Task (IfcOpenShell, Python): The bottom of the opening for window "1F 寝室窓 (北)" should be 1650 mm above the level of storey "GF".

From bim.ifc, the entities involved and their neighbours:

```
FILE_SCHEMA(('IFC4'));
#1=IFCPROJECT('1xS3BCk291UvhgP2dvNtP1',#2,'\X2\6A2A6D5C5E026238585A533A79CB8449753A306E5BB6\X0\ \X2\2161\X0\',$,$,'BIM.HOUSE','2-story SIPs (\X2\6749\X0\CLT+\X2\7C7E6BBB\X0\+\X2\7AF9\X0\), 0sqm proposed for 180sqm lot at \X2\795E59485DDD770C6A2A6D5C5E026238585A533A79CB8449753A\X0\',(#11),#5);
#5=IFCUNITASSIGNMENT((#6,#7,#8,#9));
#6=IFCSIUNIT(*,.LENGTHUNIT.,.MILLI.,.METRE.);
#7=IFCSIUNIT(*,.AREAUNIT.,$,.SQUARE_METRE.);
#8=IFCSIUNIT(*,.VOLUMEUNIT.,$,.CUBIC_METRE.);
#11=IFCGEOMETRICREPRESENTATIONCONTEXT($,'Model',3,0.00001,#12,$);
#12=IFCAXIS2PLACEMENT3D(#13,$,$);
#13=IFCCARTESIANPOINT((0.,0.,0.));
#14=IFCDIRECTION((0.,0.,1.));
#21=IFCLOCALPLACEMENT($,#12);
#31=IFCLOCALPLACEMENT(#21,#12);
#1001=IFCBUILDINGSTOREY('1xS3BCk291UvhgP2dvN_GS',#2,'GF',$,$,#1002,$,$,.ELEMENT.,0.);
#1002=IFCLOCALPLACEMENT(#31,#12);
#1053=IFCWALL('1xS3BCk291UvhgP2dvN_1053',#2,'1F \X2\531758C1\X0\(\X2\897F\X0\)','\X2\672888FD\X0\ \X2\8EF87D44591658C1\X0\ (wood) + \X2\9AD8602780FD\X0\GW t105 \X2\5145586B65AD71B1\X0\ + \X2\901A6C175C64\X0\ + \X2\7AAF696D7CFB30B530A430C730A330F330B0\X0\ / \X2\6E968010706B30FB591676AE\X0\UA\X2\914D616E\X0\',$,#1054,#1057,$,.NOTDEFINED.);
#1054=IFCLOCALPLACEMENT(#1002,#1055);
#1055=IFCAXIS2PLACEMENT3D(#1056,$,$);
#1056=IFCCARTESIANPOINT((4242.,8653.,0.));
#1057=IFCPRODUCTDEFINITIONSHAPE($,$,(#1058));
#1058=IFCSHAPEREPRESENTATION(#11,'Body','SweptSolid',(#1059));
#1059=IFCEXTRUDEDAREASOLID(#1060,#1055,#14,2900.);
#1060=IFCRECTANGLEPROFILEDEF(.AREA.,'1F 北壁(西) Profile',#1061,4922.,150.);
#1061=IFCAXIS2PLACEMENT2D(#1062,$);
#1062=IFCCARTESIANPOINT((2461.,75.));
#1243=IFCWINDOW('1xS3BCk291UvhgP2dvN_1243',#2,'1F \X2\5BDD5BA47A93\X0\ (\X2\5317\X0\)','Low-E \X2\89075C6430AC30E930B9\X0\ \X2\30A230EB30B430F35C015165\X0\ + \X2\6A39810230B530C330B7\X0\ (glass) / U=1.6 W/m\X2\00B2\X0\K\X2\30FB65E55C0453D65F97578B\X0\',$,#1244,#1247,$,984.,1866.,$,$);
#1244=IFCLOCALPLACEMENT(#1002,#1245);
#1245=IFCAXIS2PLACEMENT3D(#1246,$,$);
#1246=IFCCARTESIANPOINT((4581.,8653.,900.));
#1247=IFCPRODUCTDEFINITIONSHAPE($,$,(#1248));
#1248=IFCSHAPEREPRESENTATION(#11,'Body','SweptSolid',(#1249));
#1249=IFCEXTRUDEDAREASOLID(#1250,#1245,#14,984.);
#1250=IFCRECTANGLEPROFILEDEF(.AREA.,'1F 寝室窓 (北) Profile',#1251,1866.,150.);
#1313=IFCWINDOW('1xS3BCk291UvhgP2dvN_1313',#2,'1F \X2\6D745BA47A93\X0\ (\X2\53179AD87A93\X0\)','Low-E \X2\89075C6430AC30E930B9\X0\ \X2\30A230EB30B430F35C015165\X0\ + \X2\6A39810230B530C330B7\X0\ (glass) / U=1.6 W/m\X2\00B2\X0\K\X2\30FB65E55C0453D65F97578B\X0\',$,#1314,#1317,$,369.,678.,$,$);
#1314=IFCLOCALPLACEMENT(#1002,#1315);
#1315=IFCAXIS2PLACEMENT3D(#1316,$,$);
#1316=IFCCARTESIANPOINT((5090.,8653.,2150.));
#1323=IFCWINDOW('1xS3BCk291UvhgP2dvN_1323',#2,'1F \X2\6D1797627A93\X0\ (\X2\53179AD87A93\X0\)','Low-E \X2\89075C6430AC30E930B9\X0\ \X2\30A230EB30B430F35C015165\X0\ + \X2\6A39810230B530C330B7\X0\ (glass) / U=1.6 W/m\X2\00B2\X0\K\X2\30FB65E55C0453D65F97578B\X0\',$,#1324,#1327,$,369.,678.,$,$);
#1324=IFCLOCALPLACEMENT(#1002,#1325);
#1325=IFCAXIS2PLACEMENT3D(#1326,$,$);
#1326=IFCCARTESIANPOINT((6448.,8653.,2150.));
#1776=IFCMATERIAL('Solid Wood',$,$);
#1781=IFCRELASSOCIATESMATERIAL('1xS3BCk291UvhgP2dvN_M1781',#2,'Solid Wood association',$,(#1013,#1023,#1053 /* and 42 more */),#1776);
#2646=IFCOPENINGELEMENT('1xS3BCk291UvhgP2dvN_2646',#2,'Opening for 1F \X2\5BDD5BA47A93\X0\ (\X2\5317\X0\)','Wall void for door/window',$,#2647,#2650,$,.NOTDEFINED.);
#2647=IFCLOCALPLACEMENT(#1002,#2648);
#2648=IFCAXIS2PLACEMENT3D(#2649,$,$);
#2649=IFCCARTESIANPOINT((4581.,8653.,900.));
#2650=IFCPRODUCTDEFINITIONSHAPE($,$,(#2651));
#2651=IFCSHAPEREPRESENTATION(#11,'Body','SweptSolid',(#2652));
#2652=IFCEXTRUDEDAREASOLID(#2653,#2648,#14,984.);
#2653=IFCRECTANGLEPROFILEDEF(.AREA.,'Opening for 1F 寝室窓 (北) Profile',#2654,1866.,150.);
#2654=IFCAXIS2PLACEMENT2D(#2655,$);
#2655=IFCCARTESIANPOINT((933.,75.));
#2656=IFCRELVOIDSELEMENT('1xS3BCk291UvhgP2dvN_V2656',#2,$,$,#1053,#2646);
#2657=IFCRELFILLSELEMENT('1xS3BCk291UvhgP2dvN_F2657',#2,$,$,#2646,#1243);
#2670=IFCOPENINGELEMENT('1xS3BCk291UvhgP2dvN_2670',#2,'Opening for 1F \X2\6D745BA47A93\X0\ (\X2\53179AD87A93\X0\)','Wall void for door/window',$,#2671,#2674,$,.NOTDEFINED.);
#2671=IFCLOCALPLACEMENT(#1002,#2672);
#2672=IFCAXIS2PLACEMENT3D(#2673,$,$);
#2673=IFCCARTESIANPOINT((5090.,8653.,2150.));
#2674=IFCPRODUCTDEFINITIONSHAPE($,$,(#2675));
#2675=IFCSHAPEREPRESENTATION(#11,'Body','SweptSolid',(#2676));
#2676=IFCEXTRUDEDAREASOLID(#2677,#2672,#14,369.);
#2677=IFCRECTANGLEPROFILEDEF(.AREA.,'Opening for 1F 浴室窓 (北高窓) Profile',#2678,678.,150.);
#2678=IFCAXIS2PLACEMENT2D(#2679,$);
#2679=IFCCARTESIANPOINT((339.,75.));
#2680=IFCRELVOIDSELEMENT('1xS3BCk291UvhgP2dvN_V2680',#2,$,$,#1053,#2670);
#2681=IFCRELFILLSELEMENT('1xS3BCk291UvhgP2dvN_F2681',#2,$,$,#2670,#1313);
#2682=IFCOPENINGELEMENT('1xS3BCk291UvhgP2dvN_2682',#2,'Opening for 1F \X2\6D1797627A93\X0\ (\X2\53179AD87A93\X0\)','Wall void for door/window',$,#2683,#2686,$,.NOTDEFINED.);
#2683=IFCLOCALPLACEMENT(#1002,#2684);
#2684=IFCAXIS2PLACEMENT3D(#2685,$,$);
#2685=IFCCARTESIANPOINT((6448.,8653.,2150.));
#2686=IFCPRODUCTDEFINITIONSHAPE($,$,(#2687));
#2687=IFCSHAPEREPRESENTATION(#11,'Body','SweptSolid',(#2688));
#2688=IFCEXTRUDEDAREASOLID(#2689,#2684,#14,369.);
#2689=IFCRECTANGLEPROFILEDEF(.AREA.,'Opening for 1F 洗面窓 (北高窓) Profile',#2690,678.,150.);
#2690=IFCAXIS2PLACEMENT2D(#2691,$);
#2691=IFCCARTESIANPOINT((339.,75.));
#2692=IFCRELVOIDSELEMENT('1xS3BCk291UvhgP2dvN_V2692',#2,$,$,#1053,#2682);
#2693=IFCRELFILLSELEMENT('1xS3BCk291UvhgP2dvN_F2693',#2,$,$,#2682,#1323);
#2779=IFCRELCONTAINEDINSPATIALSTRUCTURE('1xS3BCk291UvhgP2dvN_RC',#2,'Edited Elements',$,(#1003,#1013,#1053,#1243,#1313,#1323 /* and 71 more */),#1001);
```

```python
import numpy as np
import ifcopenshell
import ifcopenshell.api.geometry
import ifcopenshell.geom
import ifcopenshell.util.element
import ifcopenshell.util.placement
import ifcopenshell.util.shape
import ifcopenshell.util.unit

model = ifcopenshell.open("bim.ifc")
unit_scale = ifcopenshell.util.unit.calculate_unit_scale(model)

window = model.by_guid("1xS3BCk291UvhgP2dvN_1243")
opening = window.FillsVoids[0].RelatingOpeningElement
storey = ifcopenshell.util.element.get_container(window, ifc_class="IfcBuildingStorey")
level = ifcopenshell.util.placement.get_local_placement(storey.ObjectPlacement)[2, 3]

# The opening's origin need not be at the sill, so measure its lowest point.
shape = ifcopenshell.geom.create_shape(ifcopenshell.geom.settings(), opening)
bottom = ifcopenshell.util.shape.get_shape_bottom_elevation(shape, shape.geometry) / unit_scale
dz = level + 1.65 / unit_scale - bottom

shift = np.array([0.0, 0.0, dz])
# The window is not placed relative to its opening, so move both.
for product in (opening, window):
    matrix = ifcopenshell.util.placement.get_local_placement(product.ObjectPlacement)
    matrix[:3, 3] += shift
    ifcopenshell.api.geometry.edit_object_placement(model, product=product, matrix=matrix, is_si=False)

print(f"moved by {dz * unit_scale:+.3f} m")

model.write("bim_v2.ifc")
```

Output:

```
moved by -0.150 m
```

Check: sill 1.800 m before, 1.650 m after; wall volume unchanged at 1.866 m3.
